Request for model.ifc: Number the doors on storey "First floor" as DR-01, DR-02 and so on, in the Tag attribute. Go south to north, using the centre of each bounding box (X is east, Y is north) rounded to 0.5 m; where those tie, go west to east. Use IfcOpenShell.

First a look at what the model holds.

```python
import ifcopenshell
import ifcopenshell.util.element
import ifcopenshell.util.placement

model = ifcopenshell.open("model.ifc")
print(model.schema)
storey = next(s for s in model.by_type("IfcBuildingStorey") if s.Name == "First floor")
doors = [e for e in ifcopenshell.util.element.get_decomposition(storey) if e.is_a("IfcDoor")]
for e in sorted(doors, key=lambda e: e.id()):
    origin = ifcopenshell.util.placement.get_local_placement(e.ObjectPlacement)[:3, 3]
    print(e.id(), e.Tag, e.Name, origin.round(2) + 0.0, sep=" | ")
```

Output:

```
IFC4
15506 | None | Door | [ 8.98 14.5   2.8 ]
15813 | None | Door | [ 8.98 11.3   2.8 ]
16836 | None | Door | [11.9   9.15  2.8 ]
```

```python
import ifcopenshell
import ifcopenshell.geom
import ifcopenshell.util.element
import ifcopenshell.util.shape

model = ifcopenshell.open("model.ifc")
settings = ifcopenshell.geom.settings()
settings.set("use-world-coords", True)


def centre(element):
    shape = ifcopenshell.geom.create_shape(settings, element)
    return ifcopenshell.util.shape.get_bbox_centroid(shape.geometry)


storey = next(s for s in model.by_type("IfcBuildingStorey") if s.Name == "First floor")
doors = [e for e in ifcopenshell.util.element.get_decomposition(storey) if e.is_a("IfcDoor")]

# Insertion points can sit at a corner or the storey origin, so sort by the geometry (in metres).
centres = {e: centre(e) for e in doors}
doors.sort(key=lambda e: (round(centres[e][1] / 0.5), centres[e][0]))

for i, e in enumerate(doors, start=1):
    number = f"DR-{i:02d}"
    e.Tag = number
    print(e.id(), number)

model.write("model_edited.ifc")
```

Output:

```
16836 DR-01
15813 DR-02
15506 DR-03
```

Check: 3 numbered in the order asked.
